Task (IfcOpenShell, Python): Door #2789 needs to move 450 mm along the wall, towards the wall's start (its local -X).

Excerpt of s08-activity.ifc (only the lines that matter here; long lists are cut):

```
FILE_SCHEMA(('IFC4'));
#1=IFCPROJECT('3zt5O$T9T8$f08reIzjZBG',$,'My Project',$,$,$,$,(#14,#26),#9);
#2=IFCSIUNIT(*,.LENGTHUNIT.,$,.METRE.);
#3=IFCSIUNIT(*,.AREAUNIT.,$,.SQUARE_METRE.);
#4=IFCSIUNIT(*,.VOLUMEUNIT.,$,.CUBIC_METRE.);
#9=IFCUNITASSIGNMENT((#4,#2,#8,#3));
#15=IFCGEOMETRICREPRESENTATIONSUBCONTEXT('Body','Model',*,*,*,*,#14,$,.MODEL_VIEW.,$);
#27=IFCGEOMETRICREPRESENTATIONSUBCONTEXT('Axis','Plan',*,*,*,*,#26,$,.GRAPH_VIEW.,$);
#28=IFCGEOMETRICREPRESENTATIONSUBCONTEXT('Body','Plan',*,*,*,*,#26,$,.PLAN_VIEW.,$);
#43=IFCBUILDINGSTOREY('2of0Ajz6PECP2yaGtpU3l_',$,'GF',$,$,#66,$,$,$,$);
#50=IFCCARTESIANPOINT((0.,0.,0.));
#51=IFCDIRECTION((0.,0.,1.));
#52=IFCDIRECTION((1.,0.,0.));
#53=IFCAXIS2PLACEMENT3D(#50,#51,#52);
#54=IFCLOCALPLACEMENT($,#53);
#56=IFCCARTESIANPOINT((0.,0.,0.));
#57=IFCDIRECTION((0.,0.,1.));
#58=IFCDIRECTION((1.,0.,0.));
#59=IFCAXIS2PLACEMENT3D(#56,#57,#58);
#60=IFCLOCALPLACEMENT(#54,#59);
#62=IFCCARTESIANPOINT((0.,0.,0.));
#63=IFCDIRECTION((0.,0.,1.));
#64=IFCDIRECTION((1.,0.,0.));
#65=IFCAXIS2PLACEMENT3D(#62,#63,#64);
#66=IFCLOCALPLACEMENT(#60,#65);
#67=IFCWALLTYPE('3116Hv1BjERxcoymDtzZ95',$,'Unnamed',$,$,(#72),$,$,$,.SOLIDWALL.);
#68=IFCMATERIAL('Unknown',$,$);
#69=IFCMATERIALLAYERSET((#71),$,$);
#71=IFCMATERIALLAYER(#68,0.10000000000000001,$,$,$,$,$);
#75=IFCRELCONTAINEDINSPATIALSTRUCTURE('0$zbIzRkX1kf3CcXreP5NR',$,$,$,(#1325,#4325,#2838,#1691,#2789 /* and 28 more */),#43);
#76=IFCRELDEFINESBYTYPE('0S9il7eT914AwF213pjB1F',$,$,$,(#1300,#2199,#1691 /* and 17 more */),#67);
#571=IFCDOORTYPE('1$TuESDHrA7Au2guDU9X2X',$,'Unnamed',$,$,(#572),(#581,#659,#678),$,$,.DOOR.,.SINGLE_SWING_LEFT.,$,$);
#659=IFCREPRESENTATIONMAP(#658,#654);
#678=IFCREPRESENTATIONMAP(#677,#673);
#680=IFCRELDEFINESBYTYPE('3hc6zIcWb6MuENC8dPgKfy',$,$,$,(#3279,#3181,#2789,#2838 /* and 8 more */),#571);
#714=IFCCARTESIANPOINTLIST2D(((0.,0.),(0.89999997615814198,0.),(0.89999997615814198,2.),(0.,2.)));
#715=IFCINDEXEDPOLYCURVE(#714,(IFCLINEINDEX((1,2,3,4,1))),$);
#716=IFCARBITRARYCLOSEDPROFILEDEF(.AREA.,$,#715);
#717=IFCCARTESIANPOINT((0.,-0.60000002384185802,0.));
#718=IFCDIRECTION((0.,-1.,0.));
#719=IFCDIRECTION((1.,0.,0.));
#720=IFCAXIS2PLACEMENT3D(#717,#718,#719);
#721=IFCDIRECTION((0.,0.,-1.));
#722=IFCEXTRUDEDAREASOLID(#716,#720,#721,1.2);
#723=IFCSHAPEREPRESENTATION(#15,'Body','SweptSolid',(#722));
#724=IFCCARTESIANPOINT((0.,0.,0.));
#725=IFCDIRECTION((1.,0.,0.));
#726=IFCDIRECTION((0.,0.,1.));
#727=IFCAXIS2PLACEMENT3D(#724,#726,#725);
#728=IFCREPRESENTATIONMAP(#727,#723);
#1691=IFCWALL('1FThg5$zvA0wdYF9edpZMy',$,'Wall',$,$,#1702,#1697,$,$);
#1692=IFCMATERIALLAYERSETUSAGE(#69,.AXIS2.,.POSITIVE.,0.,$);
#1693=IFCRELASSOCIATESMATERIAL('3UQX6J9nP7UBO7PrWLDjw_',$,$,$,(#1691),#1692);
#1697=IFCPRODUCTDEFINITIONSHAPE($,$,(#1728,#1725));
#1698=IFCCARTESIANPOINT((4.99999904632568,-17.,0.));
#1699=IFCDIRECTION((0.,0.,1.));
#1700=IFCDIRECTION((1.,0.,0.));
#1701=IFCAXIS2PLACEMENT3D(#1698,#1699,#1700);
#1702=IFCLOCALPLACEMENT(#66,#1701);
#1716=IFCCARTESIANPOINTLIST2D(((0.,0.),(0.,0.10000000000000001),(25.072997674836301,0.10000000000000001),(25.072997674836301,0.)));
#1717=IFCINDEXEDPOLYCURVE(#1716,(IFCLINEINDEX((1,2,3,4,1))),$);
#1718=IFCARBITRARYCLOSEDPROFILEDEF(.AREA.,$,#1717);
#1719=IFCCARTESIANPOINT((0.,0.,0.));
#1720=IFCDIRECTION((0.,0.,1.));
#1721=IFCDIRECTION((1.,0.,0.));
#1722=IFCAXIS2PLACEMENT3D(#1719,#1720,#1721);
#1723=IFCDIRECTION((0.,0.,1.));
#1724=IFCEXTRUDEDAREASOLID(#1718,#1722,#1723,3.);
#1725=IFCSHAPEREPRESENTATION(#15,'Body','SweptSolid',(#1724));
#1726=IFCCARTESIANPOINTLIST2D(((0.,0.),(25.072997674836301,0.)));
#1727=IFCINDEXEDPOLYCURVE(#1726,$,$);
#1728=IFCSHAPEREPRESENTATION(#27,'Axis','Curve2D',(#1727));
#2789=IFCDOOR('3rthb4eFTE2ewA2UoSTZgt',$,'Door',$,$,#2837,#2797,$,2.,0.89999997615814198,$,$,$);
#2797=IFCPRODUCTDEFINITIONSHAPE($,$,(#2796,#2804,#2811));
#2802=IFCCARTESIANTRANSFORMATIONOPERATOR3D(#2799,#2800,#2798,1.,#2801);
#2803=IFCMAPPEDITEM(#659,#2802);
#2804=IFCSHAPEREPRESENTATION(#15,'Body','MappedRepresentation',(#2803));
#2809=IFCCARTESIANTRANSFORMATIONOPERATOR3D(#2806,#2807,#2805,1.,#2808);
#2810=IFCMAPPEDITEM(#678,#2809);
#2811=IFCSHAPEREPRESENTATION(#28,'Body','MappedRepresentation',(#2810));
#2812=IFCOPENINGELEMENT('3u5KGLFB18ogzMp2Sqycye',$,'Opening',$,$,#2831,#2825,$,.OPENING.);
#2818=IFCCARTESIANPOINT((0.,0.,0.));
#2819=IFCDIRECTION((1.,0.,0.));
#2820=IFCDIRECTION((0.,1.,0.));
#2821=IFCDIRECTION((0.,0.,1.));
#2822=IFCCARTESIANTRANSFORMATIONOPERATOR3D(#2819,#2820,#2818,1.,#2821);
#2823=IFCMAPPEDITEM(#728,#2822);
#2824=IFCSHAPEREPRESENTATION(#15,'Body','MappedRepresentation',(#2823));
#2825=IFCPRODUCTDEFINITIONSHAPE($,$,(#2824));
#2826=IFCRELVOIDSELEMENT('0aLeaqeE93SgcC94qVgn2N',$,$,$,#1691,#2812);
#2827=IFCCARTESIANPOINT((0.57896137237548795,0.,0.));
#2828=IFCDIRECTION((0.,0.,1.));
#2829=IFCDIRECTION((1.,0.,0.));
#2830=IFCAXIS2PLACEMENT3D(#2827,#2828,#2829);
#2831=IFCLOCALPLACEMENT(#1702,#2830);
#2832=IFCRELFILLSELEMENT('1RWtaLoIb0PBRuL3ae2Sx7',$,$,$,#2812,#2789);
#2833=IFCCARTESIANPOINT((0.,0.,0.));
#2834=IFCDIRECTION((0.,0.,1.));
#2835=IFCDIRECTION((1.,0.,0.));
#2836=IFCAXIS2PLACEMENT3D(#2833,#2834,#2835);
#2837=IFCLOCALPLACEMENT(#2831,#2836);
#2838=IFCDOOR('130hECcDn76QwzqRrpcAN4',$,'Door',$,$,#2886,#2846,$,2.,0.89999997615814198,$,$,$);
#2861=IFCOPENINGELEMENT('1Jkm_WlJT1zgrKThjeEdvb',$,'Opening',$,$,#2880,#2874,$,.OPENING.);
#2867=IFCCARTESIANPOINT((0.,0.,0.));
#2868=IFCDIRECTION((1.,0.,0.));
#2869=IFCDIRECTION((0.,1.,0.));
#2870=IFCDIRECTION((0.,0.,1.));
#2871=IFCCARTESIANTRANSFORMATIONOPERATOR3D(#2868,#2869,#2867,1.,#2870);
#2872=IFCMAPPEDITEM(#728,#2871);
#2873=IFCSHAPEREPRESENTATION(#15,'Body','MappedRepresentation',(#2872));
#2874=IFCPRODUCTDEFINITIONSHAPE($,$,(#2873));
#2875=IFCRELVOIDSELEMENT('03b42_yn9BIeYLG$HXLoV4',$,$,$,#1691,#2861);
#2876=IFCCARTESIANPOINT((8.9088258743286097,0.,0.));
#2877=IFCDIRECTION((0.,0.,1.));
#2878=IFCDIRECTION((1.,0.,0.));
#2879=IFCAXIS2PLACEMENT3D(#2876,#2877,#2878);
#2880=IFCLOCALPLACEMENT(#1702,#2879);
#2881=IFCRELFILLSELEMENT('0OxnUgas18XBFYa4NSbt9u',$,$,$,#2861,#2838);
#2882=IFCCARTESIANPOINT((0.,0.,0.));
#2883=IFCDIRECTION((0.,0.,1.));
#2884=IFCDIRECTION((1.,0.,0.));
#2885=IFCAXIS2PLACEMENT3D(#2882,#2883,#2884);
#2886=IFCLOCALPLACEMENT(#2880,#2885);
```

```python
import ifcopenshell
import ifcopenshell.api.geometry
import ifcopenshell.util.placement
import ifcopenshell.util.unit

model = ifcopenshell.open("s08-activity.ifc")
unit_scale = ifcopenshell.util.unit.calculate_unit_scale(model)

door = model.by_guid("3rthb4eFTE2ewA2UoSTZgt")
opening = door.FillsVoids[0].RelatingOpeningElement
wall = opening.VoidsElements[0].RelatingBuildingElement

wall_matrix = ifcopenshell.util.placement.get_local_placement(wall.ObjectPlacement)
shift = wall_matrix[:3, 0] * -0.45 / unit_scale
before = ifcopenshell.util.placement.get_local_placement(door.ObjectPlacement)[:3, 3].copy()

# The door is placed relative to its opening, so it follows when the opening moves.
matrix = ifcopenshell.util.placement.get_local_placement(opening.ObjectPlacement)
matrix[:3, 3] += shift
ifcopenshell.api.geometry.edit_object_placement(
    model, product=opening, matrix=matrix, is_si=False, should_transform_children=True
)

after = ifcopenshell.util.placement.get_local_placement(door.ObjectPlacement)[:3, 3]
print("door moved by", (after - before).round(3) + 0.0)

model.write("s08-activity-out.ifc")
```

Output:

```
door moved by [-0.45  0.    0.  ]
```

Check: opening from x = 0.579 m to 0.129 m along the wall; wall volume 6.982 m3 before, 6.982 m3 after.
